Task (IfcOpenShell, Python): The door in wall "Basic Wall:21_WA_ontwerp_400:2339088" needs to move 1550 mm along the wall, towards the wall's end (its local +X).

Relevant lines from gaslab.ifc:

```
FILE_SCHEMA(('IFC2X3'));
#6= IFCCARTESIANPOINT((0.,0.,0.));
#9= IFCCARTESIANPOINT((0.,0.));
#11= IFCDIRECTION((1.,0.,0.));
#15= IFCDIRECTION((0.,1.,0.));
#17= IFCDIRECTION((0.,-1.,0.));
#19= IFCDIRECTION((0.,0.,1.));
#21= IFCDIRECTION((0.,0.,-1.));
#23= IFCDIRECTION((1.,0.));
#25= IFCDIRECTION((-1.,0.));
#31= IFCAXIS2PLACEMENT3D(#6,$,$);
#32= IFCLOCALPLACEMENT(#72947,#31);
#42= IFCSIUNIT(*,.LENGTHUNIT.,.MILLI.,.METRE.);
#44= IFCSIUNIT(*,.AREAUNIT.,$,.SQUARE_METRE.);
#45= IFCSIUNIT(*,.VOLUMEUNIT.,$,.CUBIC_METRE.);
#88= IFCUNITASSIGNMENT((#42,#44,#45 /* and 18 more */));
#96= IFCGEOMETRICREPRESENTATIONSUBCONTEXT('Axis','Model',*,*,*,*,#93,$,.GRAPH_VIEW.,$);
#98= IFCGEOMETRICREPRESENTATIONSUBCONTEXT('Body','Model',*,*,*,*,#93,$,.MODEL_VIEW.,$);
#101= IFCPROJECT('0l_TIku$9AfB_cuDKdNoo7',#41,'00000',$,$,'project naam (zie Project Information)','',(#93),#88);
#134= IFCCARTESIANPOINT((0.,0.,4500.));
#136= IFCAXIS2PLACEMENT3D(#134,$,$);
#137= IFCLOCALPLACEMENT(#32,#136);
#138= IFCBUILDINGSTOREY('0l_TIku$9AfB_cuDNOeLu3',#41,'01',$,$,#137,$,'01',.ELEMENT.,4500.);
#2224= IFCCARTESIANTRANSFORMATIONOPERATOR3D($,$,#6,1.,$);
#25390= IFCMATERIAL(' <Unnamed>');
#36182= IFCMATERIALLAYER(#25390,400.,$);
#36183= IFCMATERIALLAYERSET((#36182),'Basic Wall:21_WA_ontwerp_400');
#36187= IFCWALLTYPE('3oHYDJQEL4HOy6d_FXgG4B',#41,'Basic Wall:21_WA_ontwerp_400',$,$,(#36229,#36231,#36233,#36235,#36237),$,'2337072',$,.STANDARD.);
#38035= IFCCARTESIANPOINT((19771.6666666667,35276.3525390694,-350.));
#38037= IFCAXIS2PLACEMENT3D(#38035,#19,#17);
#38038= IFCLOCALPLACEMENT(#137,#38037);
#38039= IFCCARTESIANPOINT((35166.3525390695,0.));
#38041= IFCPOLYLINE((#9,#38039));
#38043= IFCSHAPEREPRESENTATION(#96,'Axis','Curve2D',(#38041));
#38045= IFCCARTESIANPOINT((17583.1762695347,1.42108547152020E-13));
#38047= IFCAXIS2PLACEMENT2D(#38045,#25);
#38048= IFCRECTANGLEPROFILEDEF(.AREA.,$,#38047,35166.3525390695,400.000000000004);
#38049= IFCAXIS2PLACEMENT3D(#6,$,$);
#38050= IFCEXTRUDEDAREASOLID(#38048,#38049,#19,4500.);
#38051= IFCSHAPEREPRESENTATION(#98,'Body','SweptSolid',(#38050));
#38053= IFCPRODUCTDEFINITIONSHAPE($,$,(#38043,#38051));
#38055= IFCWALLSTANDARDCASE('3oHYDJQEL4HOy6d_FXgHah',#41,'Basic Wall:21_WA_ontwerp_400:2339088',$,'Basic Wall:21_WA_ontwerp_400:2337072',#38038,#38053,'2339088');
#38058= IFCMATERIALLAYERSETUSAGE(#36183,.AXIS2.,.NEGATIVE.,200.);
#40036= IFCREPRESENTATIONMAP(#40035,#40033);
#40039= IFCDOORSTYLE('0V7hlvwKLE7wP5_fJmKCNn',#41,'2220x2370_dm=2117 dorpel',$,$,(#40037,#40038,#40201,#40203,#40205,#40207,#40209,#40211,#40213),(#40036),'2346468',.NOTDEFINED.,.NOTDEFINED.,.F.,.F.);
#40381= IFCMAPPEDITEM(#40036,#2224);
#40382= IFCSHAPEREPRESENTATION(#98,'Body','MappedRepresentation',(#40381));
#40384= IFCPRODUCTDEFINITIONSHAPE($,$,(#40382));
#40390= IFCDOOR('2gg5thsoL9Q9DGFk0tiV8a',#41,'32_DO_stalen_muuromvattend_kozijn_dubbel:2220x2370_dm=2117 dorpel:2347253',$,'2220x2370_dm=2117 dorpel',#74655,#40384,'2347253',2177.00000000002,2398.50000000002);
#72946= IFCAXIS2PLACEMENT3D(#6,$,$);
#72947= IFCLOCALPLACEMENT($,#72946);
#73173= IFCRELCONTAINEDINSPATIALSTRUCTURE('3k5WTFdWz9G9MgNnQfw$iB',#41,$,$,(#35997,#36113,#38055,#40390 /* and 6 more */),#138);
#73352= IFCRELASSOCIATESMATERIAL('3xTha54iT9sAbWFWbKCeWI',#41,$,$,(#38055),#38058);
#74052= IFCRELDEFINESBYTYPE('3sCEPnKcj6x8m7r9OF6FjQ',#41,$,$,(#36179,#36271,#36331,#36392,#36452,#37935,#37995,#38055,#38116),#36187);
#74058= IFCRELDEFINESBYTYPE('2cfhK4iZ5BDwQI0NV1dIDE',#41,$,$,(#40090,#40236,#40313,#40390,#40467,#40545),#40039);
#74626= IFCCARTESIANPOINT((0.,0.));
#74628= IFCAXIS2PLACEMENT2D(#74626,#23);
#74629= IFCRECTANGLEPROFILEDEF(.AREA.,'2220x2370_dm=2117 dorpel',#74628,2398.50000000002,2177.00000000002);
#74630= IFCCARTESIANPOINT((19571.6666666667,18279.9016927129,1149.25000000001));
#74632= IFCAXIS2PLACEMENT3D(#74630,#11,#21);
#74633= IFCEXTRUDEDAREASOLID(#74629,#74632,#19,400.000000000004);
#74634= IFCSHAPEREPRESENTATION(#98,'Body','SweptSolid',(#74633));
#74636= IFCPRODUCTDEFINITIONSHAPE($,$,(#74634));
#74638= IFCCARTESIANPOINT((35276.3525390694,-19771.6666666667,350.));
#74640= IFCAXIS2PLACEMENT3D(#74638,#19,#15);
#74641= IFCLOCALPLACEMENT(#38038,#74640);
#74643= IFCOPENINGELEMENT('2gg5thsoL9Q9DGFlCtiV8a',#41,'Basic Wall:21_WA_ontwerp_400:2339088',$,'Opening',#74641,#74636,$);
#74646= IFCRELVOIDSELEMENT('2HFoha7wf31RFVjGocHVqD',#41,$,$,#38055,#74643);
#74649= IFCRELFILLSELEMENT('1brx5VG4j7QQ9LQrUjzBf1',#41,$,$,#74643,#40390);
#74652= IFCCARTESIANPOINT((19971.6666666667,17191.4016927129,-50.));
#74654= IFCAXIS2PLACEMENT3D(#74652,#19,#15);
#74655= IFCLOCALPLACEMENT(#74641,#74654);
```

```python
import ifcopenshell
import ifcopenshell.api.geometry
import ifcopenshell.util.placement
import ifcopenshell.util.unit

model = ifcopenshell.open("gaslab.ifc")
unit_scale = ifcopenshell.util.unit.calculate_unit_scale(model)

door = model.by_guid("2gg5thsoL9Q9DGFk0tiV8a")
opening = door.FillsVoids[0].RelatingOpeningElement
wall = opening.VoidsElements[0].RelatingBuildingElement

wall_matrix = ifcopenshell.util.placement.get_local_placement(wall.ObjectPlacement)
shift = wall_matrix[:3, 0] * 1.55 / unit_scale
before = ifcopenshell.util.placement.get_local_placement(door.ObjectPlacement)[:3, 3].copy()

# The door is placed relative to its opening, so it follows when the opening moves.
matrix = ifcopenshell.util.placement.get_local_placement(opening.ObjectPlacement)
matrix[:3, 3] += shift
ifcopenshell.api.geometry.edit_object_placement(
    model, product=opening, matrix=matrix, is_si=False, should_transform_children=True
)

after = ifcopenshell.util.placement.get_local_placement(door.ObjectPlacement)[:3, 3]
print("door moved by", (after - before).round(3) + 0.0)

model.write("gaslab_edited.ifc")
```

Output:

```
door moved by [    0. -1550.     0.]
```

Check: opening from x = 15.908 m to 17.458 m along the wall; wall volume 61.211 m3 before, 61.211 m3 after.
